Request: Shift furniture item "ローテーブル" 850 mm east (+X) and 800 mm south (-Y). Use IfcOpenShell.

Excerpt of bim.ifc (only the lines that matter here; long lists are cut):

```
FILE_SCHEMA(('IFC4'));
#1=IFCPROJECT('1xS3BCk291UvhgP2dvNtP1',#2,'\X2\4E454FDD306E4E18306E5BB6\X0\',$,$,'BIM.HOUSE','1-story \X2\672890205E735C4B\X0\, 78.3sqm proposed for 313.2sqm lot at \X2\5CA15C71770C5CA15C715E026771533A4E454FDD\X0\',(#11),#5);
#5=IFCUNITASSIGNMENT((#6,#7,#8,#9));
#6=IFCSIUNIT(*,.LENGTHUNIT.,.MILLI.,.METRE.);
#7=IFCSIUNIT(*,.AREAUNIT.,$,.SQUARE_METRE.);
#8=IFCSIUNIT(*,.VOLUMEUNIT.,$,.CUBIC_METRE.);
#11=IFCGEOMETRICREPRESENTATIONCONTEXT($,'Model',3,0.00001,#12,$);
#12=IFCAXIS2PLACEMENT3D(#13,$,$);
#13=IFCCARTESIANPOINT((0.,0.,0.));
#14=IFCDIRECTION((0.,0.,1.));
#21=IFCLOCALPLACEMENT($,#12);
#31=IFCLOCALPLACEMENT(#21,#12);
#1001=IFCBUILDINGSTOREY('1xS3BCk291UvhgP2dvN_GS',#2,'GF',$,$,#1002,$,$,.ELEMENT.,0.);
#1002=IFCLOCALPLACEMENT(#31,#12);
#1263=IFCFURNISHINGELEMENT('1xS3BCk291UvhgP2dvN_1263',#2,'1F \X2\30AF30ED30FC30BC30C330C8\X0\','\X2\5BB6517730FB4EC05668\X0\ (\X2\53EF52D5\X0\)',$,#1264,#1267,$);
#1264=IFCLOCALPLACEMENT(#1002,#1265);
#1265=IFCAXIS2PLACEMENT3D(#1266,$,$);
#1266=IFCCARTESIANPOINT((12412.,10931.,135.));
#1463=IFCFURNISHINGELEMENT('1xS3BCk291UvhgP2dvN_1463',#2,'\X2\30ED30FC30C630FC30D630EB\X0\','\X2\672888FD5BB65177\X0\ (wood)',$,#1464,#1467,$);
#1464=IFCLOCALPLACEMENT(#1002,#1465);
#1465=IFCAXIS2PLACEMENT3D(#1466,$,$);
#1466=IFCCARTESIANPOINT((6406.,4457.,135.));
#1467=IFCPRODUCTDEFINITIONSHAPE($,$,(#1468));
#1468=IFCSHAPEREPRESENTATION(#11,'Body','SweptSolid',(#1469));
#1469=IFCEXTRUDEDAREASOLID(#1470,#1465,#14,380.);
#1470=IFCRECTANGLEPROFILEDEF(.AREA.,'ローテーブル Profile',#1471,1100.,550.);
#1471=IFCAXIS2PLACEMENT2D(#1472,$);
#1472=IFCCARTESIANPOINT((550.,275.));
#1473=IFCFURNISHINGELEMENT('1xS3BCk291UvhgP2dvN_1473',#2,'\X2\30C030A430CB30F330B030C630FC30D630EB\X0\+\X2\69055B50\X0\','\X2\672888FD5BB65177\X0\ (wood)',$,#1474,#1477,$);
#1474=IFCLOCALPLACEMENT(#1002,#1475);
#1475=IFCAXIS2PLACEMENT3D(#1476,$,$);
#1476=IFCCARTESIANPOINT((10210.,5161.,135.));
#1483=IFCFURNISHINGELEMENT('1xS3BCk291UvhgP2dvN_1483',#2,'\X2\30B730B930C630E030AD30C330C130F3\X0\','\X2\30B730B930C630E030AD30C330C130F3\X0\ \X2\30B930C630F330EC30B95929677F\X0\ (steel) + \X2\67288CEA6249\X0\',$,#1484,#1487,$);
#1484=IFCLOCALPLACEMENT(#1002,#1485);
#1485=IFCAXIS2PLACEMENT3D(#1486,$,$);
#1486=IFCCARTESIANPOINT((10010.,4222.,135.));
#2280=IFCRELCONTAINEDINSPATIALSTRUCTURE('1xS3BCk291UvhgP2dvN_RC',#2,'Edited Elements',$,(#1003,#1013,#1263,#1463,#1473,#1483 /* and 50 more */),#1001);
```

```python
import ifcopenshell
import ifcopenshell.api.geometry
import ifcopenshell.util.placement

model = ifcopenshell.open("bim.ifc")

item = model.by_guid("1xS3BCk291UvhgP2dvN_1463")
matrix = ifcopenshell.util.placement.get_local_placement(item.ObjectPlacement)
matrix[0, 3] += 850.0
matrix[1, 3] -= 800.0
ifcopenshell.api.geometry.edit_object_placement(model, product=item, matrix=matrix, is_si=False)

print(ifcopenshell.util.placement.get_local_placement(item.ObjectPlacement).round(3) + 0.0)

model.write("bim_rev.ifc")
```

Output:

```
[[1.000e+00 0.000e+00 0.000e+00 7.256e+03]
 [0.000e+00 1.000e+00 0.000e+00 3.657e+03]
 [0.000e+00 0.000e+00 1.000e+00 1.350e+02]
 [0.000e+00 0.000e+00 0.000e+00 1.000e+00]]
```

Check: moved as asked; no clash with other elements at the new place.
